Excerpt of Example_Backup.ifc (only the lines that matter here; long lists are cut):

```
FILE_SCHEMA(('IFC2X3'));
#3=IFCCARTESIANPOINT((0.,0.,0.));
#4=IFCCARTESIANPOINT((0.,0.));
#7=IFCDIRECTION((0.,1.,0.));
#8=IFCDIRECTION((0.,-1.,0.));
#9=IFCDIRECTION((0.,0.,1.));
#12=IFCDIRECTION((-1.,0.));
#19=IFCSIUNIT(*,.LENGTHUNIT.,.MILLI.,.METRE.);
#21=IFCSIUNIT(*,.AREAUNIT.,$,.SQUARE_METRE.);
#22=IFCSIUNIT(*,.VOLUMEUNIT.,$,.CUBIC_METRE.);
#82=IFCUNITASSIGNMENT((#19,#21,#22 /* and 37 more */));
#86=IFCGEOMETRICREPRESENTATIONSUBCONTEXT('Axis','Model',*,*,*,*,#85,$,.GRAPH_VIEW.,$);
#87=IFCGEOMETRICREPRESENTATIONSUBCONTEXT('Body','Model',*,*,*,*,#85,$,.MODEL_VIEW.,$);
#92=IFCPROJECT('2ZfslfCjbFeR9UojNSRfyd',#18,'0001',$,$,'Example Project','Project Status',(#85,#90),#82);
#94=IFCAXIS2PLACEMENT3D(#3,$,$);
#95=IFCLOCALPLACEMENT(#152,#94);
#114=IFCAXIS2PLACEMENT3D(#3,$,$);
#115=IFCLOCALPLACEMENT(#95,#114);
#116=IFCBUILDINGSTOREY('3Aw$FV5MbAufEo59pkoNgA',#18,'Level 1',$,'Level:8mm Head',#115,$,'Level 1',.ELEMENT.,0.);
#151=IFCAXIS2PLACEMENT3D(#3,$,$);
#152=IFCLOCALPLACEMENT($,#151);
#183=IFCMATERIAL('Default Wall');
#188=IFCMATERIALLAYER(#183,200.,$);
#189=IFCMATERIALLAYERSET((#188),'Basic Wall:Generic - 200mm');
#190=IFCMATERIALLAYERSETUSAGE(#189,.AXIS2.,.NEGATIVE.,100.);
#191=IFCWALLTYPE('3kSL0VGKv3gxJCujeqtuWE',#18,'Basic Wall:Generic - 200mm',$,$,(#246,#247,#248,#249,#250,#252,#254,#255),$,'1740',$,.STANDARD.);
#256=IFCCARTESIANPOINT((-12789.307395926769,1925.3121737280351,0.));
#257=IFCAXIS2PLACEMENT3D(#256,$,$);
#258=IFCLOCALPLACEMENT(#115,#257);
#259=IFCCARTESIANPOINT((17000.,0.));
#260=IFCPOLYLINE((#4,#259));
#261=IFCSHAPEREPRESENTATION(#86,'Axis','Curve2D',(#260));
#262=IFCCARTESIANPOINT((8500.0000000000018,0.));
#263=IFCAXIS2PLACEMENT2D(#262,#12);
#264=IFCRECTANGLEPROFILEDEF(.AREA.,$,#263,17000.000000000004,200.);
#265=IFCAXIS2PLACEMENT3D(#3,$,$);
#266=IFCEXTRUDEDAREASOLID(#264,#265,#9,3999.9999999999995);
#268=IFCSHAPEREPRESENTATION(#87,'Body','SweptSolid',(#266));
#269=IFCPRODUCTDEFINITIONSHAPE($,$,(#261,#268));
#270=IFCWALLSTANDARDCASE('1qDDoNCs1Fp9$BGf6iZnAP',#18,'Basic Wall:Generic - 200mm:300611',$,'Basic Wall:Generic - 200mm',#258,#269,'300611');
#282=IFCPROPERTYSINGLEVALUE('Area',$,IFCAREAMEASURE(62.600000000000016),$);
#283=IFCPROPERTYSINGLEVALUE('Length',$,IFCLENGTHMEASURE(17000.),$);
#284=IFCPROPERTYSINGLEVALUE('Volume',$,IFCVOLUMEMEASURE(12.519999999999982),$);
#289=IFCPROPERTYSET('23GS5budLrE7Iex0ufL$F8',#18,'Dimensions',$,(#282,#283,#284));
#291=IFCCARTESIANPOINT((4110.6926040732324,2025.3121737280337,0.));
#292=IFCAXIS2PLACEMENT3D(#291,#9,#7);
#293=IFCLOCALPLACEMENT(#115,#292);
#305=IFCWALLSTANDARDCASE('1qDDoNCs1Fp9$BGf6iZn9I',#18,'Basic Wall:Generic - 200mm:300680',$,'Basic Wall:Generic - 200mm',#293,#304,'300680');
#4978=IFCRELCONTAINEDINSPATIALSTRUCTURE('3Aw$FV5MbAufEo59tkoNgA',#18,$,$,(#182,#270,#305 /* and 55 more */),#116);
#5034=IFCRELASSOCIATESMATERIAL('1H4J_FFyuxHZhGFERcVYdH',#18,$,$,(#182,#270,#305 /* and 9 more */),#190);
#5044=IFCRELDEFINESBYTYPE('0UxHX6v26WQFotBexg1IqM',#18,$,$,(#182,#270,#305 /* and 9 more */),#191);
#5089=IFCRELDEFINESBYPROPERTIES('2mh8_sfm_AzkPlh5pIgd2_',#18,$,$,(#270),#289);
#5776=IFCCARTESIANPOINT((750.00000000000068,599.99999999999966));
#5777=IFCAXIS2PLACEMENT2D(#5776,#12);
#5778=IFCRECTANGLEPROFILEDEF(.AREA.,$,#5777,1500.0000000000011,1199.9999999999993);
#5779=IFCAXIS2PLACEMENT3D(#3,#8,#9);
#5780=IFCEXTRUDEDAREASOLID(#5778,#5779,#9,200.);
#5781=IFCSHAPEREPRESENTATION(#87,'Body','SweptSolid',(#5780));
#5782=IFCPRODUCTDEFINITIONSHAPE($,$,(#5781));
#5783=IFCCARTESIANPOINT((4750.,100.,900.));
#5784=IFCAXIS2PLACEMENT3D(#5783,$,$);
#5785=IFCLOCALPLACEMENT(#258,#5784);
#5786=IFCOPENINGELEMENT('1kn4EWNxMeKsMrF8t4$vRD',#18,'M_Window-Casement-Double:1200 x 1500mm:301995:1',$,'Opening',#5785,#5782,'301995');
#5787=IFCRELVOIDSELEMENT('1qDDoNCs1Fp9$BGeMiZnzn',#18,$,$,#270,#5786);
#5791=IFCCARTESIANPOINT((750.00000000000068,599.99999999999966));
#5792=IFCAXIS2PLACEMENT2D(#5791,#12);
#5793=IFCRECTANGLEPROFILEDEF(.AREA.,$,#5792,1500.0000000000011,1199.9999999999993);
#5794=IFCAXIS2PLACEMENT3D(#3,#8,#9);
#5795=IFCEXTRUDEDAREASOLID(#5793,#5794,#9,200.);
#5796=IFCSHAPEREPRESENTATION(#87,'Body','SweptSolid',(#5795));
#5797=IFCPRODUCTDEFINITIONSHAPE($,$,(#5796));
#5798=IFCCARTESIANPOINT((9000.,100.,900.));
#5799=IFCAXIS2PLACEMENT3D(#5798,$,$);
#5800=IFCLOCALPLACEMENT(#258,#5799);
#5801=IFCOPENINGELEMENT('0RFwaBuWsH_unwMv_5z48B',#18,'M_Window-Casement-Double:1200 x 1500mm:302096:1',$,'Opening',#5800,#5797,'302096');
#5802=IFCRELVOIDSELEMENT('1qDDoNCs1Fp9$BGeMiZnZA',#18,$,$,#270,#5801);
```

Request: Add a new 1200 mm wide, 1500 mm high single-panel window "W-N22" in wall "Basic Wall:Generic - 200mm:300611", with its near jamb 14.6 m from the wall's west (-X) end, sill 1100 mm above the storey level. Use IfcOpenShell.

```python
import numpy as np
import ifcopenshell
import ifcopenshell.api.feature
import ifcopenshell.api.geometry
import ifcopenshell.api.pset
import ifcopenshell.api.root
import ifcopenshell.api.spatial
import ifcopenshell.api.type
import ifcopenshell.geom
import ifcopenshell.util.element
import ifcopenshell.util.placement
import ifcopenshell.util.representation
import ifcopenshell.util.shape
import ifcopenshell.util.unit

model = ifcopenshell.open("Example_Backup.ifc")
unit_scale = ifcopenshell.util.unit.calculate_unit_scale(model)
area_scale = ifcopenshell.util.unit.calculate_unit_scale(model, "AREAUNIT")
volume_scale = ifcopenshell.util.unit.calculate_unit_scale(model, "VOLUMEUNIT")
settings = ifcopenshell.geom.settings()


def volume(element):
    """Net volume in cubic metres, openings subtracted."""
    shape = ifcopenshell.geom.create_shape(settings, element)
    return ifcopenshell.util.shape.get_volume(shape.geometry)


wall = model.by_id(270)
storey = ifcopenshell.util.element.get_container(wall, ifc_class="IfcBuildingStorey")
context = ifcopenshell.util.representation.get_context(model, "Model", "Body", "MODEL_VIEW")
before = volume(wall)

width, height, from_end, sill = 1.2, 1.5, 14.6, 1.1  # metres

# The wall runs along its own X axis, and the end named is its -X end.
wall_shape = ifcopenshell.geom.create_shape(settings, wall)
x, y, z = ifcopenshell.util.shape.get_vertices(wall_shape.geometry).T
start = x.min() + from_end
face, thickness = float(y.min()), float(y.max() - y.min())
wall_matrix = ifcopenshell.util.placement.get_local_placement(wall.ObjectPlacement)
level = ifcopenshell.util.placement.get_local_placement(storey.ObjectPlacement)[2, 3]


def in_wall(x, y):
    """Placement at x, y metres in the wall's axes, at sill height."""
    matrix = wall_matrix.copy()
    matrix[:, 3] = wall_matrix @ np.array([x / unit_scale, y / unit_scale, 0.0, 1.0])
    matrix[2, 3] = level + sill / unit_scale
    return matrix


# Opening: a box that overshoots both wall faces by 50 mm.
opening = ifcopenshell.api.root.create_entity(model, ifc_class="IfcOpeningElement")
box = ifcopenshell.api.geometry.add_wall_representation(
    model, context=context, length=width, height=height, thickness=thickness + 0.1
)
ifcopenshell.api.geometry.assign_representation(model, product=opening, representation=box)
ifcopenshell.api.geometry.edit_object_placement(model, product=opening, matrix=in_wall(start, face - 0.05), is_si=False)
ifcopenshell.api.feature.add_feature(model, feature=opening, element=wall)

window = ifcopenshell.api.root.create_entity(model, ifc_class="IfcWindow", name="W-N22")
window.OverallWidth, window.OverallHeight = width / unit_scale, height / unit_scale
body = ifcopenshell.api.geometry.add_window_representation(
    model,
    context=context,
    overall_width=window.OverallWidth,
    overall_height=window.OverallHeight,
    partition_type="SINGLE_PANEL",
)
ifcopenshell.api.geometry.assign_representation(model, product=window, representation=body)
ifcopenshell.api.spatial.assign_container(model, products=[window], relating_structure=storey)
fills = ifcopenshell.api.feature.add_filling(model, opening=opening, element=window)
fills.OwnerHistory = window.OwnerHistory  # required in IFC2X3

# IFC2X3 keeps the operation on the window style.
style = ifcopenshell.api.root.create_entity(model, ifc_class="IfcWindowStyle", name="W-N22")
style.OperationType, style.ConstructionType = "SINGLE_PANEL", "NOTDEFINED"
style.ParameterTakesPrecedence = style.Sizeable = False
ifcopenshell.api.type.assign_type(model, related_objects=[window], relating_type=style)

# Centre the window in the wall's thickness.
ifcopenshell.api.geometry.edit_object_placement(model, product=window, matrix=in_wall(start, face), is_si=False)
window_shape = ifcopenshell.geom.create_shape(settings, window)
depth = ifcopenshell.util.shape.get_vertices(window_shape.geometry)[:, 1]
offset = face + thickness / 2 - (depth.min() + depth.max()) / 2
ifcopenshell.api.geometry.edit_object_placement(model, product=window, matrix=in_wall(start, offset), is_si=False)

after = volume(wall)

# Update the wall's stored quantities.
pset = model.by_id(ifcopenshell.util.element.get_pset(wall, "Dimensions", should_inherit=False)["id"])
ifcopenshell.api.pset.edit_pset(model, pset=pset, properties={
    "Area": model.create_entity("IfcAreaMeasure", after / thickness / area_scale),
    "Volume": model.create_entity("IfcVolumeMeasure", after / volume_scale),
})

print(f"wall volume {before:.3f} -> {after:.3f} m3")

model.write("Example_Backup_edited.ifc")
```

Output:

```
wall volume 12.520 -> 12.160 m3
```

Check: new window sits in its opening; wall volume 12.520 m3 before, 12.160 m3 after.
